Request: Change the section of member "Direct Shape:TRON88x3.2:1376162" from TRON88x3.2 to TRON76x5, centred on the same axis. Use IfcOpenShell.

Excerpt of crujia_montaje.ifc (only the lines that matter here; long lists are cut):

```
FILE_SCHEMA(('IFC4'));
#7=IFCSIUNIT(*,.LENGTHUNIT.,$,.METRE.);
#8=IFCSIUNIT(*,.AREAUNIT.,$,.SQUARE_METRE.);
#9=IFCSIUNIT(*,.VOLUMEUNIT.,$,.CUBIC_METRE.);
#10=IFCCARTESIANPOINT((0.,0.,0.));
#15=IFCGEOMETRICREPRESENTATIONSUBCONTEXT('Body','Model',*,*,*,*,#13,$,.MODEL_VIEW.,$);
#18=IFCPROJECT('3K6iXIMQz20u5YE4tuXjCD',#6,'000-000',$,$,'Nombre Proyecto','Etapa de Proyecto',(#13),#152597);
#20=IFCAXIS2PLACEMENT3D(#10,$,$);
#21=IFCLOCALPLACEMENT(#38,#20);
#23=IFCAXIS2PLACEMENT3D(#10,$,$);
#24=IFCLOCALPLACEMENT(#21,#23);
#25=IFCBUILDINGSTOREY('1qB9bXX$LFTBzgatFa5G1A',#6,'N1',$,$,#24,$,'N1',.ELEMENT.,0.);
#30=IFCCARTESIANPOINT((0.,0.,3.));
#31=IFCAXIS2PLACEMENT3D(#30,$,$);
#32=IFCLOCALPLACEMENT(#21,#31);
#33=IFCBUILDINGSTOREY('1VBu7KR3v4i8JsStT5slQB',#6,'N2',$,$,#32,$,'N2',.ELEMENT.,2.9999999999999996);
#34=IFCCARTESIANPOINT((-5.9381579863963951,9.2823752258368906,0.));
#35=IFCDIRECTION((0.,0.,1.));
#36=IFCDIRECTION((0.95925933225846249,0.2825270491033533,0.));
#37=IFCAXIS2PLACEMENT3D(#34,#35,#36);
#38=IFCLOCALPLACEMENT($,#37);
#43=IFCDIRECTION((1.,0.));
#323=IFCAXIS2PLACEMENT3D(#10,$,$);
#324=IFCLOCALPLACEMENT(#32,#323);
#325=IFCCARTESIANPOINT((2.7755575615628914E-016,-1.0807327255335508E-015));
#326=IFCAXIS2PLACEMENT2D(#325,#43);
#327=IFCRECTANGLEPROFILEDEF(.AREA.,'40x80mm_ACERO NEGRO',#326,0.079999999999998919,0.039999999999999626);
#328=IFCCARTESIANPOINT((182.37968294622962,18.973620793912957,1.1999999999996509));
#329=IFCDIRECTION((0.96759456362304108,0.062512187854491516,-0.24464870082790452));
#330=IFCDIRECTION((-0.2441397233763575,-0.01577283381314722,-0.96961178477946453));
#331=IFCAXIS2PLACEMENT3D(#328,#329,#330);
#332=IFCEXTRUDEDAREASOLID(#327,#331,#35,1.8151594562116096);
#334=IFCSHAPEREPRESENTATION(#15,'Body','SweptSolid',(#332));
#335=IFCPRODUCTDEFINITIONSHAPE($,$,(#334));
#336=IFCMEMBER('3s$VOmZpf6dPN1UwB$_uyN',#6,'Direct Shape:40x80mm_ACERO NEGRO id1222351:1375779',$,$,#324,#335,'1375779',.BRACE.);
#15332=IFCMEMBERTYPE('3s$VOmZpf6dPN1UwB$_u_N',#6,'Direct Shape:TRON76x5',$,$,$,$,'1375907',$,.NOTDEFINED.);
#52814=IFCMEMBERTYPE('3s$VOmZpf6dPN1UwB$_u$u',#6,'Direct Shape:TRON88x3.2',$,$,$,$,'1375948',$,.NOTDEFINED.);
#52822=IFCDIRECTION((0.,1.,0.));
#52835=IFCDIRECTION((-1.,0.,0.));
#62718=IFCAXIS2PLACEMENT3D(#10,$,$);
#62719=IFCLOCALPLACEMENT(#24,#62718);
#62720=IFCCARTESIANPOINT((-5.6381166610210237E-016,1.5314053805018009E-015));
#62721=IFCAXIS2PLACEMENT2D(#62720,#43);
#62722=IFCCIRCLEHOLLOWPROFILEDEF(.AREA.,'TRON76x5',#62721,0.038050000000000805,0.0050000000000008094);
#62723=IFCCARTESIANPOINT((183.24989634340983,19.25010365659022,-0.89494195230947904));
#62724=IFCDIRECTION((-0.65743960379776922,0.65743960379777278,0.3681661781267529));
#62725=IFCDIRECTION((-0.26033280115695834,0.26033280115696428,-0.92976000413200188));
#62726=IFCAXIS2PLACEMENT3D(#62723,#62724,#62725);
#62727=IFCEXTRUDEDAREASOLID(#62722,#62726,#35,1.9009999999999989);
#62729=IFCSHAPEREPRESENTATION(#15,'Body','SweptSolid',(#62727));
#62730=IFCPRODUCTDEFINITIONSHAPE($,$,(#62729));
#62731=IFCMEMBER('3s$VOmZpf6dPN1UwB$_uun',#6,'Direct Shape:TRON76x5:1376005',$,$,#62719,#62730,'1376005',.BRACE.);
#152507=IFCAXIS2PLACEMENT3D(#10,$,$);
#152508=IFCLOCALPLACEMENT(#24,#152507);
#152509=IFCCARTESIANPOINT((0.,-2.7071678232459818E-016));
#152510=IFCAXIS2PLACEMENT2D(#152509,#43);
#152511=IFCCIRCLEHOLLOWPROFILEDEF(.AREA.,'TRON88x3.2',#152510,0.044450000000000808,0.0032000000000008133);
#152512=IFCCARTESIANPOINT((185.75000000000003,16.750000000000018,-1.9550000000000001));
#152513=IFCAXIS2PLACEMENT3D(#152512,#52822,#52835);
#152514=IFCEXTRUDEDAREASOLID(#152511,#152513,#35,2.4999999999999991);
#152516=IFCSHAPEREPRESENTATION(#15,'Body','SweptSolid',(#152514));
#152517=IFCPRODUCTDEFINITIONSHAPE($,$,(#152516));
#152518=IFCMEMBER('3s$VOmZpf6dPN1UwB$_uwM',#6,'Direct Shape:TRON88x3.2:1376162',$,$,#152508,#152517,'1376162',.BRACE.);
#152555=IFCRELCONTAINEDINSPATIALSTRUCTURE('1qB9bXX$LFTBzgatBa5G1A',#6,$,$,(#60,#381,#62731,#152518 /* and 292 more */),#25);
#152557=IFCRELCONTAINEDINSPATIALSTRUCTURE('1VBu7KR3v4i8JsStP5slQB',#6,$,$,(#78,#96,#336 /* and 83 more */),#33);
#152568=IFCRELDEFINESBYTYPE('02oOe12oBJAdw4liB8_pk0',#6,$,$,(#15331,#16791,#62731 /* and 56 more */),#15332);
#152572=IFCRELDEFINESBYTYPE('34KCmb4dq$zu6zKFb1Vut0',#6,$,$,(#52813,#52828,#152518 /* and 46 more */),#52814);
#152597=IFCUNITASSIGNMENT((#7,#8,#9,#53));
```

```python
import ifcopenshell
import ifcopenshell.api.type
import ifcopenshell.util.element
import ifcopenshell.util.representation

model = ifcopenshell.open("crujia_montaje.ifc")

member = model.by_guid("3s$VOmZpf6dPN1UwB$_uwM")
source = next(p for p in model.by_type("IfcCircleHollowProfileDef") if p.ProfileName == "TRON76x5")

body = ifcopenshell.util.representation.get_representation(member, "Model", "Body")
solid = body.Items[0]
old_profile = solid.SweptArea

# Copy the section's sizes but keep this member's own profile position.
profile = ifcopenshell.util.element.copy(model, source)
profile.Position = old_profile.Position
solid.SweptArea = profile
if not model.get_total_inverses(old_profile):
    ifcopenshell.util.element.remove_deep2(model, old_profile)

new_type = model.by_guid("3s$VOmZpf6dPN1UwB$_u_N")
ifcopenshell.api.type.assign_type(
    model, related_objects=[member], relating_type=new_type, should_map_representations=False
)
member.Name = member.Name.replace("TRON88x3.2", "TRON76x5")

print(solid.SweptArea)

model.write("crujia_montaje_rev.ifc")
```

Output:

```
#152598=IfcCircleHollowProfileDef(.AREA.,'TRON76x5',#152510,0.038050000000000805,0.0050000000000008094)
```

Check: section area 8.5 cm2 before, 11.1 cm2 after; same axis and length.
